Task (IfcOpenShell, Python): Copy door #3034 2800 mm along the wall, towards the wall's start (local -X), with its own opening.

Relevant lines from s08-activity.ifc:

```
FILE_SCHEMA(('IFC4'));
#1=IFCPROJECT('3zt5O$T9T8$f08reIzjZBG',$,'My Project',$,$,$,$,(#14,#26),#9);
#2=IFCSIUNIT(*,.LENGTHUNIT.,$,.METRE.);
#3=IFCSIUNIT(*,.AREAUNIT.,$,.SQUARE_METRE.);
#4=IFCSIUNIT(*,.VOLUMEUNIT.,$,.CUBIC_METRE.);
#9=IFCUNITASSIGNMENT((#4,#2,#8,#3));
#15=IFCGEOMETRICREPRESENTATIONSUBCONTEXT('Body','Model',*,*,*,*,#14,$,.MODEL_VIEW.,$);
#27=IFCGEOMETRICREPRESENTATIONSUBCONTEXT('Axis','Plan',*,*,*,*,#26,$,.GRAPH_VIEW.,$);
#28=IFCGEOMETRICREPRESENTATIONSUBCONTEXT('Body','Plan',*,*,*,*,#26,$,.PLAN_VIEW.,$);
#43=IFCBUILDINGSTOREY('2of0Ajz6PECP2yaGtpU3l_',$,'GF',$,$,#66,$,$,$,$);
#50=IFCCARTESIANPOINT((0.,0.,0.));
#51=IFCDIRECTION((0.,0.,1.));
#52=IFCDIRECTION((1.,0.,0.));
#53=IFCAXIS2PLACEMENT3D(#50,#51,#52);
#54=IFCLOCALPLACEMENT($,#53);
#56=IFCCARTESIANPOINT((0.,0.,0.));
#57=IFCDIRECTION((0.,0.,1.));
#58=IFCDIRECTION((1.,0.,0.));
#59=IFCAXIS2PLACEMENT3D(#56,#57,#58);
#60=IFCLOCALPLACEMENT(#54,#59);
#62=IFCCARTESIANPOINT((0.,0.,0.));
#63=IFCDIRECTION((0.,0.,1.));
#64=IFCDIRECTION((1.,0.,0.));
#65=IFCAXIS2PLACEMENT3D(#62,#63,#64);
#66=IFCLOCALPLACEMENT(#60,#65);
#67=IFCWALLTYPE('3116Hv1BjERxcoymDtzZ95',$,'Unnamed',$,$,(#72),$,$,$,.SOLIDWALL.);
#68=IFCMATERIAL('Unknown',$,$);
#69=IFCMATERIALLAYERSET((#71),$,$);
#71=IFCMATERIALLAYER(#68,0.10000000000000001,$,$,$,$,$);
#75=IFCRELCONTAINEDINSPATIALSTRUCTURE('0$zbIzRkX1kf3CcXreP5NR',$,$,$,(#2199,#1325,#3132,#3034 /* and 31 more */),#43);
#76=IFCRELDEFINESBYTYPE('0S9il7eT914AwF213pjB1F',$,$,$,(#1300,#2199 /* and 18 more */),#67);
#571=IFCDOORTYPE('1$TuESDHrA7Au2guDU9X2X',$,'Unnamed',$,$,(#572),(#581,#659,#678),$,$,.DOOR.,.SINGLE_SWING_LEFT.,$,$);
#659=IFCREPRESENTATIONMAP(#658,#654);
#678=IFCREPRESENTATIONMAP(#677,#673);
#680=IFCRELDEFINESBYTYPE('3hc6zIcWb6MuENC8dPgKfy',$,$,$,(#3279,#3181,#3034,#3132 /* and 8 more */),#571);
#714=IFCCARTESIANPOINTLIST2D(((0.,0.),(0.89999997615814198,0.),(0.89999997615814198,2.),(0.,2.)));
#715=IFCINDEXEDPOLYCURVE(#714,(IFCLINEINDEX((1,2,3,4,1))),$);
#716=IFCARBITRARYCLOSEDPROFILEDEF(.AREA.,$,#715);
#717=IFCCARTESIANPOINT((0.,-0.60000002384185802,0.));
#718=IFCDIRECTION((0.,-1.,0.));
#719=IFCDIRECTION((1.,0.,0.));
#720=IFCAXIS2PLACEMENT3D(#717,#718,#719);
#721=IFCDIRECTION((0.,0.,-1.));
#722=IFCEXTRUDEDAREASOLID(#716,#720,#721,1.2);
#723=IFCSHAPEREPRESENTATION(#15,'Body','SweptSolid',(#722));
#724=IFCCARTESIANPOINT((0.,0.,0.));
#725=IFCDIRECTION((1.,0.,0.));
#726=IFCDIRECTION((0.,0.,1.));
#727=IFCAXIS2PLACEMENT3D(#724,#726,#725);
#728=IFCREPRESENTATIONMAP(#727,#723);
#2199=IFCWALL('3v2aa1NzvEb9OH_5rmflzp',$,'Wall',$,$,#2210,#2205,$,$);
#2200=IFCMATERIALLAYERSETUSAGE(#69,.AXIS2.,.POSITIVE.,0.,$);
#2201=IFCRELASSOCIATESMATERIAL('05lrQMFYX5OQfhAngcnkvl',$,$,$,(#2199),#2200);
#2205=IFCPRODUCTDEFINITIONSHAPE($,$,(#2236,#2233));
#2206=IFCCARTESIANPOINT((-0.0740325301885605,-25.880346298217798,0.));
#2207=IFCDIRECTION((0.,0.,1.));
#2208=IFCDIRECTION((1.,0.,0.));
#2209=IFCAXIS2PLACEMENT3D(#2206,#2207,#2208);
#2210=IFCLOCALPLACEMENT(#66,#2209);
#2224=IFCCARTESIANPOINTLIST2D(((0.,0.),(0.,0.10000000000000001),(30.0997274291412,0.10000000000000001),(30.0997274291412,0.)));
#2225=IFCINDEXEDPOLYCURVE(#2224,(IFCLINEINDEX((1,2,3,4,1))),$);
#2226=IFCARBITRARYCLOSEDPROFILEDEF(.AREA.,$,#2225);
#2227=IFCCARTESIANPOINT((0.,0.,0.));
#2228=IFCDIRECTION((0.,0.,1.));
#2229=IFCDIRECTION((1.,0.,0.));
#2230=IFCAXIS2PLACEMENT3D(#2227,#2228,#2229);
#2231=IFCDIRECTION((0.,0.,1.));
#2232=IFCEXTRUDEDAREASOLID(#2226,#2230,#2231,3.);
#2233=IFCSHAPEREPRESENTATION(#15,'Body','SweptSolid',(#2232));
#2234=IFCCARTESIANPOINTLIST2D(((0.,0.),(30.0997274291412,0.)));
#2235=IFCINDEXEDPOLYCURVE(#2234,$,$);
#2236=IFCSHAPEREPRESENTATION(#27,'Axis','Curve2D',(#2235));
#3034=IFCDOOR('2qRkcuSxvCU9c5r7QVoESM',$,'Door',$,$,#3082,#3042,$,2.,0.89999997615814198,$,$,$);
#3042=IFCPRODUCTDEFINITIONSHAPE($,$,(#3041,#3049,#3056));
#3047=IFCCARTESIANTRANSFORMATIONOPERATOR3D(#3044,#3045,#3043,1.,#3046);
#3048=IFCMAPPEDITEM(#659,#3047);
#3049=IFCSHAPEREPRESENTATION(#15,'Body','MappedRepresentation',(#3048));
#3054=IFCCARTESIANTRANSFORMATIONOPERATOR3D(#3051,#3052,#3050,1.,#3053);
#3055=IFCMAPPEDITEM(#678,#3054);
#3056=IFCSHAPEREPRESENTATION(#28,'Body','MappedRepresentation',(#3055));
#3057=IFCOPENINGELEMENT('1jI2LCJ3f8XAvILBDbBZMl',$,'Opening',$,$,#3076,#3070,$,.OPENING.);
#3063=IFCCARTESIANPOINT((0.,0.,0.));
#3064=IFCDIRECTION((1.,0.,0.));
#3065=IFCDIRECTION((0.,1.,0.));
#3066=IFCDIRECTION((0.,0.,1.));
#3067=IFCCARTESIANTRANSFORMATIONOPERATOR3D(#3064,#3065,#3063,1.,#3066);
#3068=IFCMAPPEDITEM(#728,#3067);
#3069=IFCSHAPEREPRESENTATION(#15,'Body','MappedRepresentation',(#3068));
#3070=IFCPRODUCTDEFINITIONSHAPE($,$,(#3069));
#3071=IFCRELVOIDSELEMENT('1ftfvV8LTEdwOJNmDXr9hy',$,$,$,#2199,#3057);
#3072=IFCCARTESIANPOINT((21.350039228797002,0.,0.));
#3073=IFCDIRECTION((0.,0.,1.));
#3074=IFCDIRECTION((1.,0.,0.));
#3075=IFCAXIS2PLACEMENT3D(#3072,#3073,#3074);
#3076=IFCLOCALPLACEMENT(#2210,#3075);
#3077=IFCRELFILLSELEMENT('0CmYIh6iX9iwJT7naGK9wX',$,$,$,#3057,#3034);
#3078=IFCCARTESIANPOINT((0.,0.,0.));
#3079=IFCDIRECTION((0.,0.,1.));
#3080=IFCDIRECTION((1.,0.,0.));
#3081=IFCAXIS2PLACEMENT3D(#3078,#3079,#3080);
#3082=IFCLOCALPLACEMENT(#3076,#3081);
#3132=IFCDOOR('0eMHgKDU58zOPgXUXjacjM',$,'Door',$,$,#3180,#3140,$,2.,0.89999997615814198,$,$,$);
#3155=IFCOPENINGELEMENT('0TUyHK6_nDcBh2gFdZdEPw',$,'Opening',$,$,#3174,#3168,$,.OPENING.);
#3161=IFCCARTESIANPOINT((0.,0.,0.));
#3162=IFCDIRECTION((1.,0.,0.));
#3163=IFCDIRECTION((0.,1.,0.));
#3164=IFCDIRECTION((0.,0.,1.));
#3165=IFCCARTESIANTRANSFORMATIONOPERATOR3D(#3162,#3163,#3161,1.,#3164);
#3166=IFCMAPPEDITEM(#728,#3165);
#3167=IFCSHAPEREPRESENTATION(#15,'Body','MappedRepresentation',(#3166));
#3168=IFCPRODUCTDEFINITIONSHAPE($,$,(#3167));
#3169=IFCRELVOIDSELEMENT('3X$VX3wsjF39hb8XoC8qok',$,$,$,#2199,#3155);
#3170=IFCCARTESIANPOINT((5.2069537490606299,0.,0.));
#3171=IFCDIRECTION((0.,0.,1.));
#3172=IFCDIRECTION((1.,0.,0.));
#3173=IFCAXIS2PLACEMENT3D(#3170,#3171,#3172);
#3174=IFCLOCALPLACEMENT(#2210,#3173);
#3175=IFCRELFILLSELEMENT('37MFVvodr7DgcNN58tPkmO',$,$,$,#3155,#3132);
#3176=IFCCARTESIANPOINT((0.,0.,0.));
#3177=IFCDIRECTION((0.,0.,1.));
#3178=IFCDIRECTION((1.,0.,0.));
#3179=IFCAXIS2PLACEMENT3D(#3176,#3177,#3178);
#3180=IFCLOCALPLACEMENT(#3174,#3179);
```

```python
import ifcopenshell
import ifcopenshell.api.feature
import ifcopenshell.api.geometry
import ifcopenshell.api.root
import ifcopenshell.geom
import ifcopenshell.util.element
import ifcopenshell.util.placement
import ifcopenshell.util.shape
import ifcopenshell.util.unit

model = ifcopenshell.open("s08-activity.ifc")
unit_scale = ifcopenshell.util.unit.calculate_unit_scale(model)
settings = ifcopenshell.geom.settings()


def volume(element):
    """Net volume in cubic metres, openings subtracted."""
    shape = ifcopenshell.geom.create_shape(settings, element)
    return ifcopenshell.util.shape.get_volume(shape.geometry)


door = model.by_guid("2qRkcuSxvCU9c5r7QVoESM")
opening = door.FillsVoids[0].RelatingOpeningElement
wall = opening.VoidsElements[0].RelatingBuildingElement
before = volume(wall)
shift = ifcopenshell.util.placement.get_local_placement(wall.ObjectPlacement)[:3, 0] * -2.8 / unit_scale

# copy_class copies the void relationship, type, container and properties, but no geometry.
new_opening = ifcopenshell.api.root.copy_class(model, product=opening)
new_opening.Representation = ifcopenshell.util.element.copy_deep(
    model, opening.Representation, exclude=["IfcGeometricRepresentationContext", "IfcRepresentationMap"]
)
new_door = ifcopenshell.api.root.copy_class(model, product=door)
new_door.Representation = ifcopenshell.util.element.copy_deep(
    model, door.Representation, exclude=["IfcGeometricRepresentationContext", "IfcRepresentationMap"]
)
ifcopenshell.api.feature.add_filling(model, opening=new_opening, element=new_door)

for old, new in ((opening, new_opening), (door, new_door)):
    matrix = ifcopenshell.util.placement.get_local_placement(old.ObjectPlacement)
    matrix[:3, 3] += shift
    ifcopenshell.api.geometry.edit_object_placement(model, product=new, matrix=matrix, is_si=False)

after = volume(wall)

print(f"wall volume {before:.3f} -> {after:.3f} m3")

model.write("s08-activity-out.ifc")
```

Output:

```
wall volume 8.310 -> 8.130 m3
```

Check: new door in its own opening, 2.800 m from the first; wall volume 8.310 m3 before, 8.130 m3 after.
